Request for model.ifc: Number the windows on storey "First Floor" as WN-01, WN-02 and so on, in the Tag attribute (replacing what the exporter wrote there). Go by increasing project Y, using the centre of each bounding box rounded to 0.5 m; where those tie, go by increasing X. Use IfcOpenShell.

First a look at what the model holds.

```python
import ifcopenshell
import ifcopenshell.util.element
import ifcopenshell.util.placement

model = ifcopenshell.open("model.ifc")
print(model.schema)
storey = next(s for s in model.by_type("IfcBuildingStorey") if s.Name == "First Floor")
windows = [e for e in ifcopenshell.util.element.get_decomposition(storey) if e.is_a("IfcWindow")]
for e in sorted(windows, key=lambda e: e.id()):
    origin = ifcopenshell.util.placement.get_local_placement(e.ObjectPlacement)[:3, 3]
    print(e.id(), e.Tag, e.Name, origin.round(2) + 0.0, sep=" | ")
```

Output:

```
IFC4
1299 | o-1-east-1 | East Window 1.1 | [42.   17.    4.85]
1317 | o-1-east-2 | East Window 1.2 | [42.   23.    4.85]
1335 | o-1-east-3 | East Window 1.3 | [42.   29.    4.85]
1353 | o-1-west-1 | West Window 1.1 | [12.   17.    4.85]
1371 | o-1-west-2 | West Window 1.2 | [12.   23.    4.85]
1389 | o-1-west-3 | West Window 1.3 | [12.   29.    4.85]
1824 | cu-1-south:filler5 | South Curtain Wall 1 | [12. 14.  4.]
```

```python
import ifcopenshell
import ifcopenshell.geom
import ifcopenshell.util.element
import ifcopenshell.util.shape

model = ifcopenshell.open("model.ifc")
settings = ifcopenshell.geom.settings()
settings.set("use-world-coords", True)


def centre(element):
    shape = ifcopenshell.geom.create_shape(settings, element)
    return ifcopenshell.util.shape.get_bbox_centroid(shape.geometry)


storey = next(s for s in model.by_type("IfcBuildingStorey") if s.Name == "First Floor")
windows = [e for e in ifcopenshell.util.element.get_decomposition(storey) if e.is_a("IfcWindow")]

# Insertion points can sit at a corner or the storey origin, so sort by the geometry (in metres).
centres = {e: centre(e) for e in windows}
windows.sort(key=lambda e: (round(centres[e][1] / 0.5), centres[e][0]))

for i, e in enumerate(windows, start=1):
    number = f"WN-{i:02d}"
    e.Tag = number
    print(e.id(), number)

model.write("model_v2.ifc")
```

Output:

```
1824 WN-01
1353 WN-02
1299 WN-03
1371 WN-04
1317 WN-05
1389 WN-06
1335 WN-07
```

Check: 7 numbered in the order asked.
